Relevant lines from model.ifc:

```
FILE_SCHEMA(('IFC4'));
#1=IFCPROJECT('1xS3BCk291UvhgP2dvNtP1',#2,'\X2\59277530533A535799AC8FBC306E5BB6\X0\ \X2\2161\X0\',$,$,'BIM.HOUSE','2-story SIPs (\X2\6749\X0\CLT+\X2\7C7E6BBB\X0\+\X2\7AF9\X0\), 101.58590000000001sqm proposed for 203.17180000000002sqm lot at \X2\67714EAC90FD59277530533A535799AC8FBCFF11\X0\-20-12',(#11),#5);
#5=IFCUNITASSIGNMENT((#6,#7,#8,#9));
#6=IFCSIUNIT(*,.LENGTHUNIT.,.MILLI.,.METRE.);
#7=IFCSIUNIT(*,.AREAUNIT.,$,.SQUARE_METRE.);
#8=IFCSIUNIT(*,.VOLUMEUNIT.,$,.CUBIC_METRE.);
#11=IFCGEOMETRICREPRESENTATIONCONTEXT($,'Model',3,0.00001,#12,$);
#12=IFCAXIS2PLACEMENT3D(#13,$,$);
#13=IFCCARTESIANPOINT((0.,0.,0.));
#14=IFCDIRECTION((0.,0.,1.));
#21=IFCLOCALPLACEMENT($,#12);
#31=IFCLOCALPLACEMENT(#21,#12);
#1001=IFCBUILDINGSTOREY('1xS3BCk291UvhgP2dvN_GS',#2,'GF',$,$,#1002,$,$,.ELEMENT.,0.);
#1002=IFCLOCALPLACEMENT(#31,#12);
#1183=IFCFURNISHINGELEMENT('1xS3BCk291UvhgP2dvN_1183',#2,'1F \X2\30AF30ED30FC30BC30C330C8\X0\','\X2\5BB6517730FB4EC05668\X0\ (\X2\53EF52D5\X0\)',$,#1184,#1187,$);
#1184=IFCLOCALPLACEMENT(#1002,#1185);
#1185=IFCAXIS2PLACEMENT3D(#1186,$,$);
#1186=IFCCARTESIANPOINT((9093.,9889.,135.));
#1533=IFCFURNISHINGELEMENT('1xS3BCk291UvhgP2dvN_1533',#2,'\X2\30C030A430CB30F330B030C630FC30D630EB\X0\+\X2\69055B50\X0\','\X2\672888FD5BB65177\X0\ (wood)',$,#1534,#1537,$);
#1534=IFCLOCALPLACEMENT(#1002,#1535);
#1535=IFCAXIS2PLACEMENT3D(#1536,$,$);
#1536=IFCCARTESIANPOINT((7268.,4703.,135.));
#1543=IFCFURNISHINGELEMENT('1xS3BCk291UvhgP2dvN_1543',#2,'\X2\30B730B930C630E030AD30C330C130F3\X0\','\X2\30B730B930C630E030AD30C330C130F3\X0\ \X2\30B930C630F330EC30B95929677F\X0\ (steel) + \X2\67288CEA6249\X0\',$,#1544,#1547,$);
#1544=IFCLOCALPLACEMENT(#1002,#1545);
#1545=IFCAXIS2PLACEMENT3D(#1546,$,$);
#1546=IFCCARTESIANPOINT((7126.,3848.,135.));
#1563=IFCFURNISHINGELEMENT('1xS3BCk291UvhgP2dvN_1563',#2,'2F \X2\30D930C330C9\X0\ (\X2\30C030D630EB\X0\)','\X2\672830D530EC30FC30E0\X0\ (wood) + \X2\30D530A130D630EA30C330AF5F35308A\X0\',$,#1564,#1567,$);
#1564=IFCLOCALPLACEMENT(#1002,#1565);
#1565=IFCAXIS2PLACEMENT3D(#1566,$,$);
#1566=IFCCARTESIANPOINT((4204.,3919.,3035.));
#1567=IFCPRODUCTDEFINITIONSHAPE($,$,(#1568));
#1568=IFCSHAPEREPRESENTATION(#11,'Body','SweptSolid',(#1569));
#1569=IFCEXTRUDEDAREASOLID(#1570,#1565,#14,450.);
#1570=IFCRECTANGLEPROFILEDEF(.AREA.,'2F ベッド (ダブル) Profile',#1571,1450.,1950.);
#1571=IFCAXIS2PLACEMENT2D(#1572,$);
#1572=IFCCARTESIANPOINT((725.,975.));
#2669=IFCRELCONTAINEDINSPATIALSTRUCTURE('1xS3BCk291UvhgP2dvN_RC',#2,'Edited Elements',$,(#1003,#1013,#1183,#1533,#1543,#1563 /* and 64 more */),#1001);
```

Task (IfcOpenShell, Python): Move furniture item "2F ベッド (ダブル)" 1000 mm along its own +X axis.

```python
import ifcopenshell
import ifcopenshell.api.geometry
import ifcopenshell.util.placement

model = ifcopenshell.open("model.ifc")

item = model.by_guid("1xS3BCk291UvhgP2dvN_1563")
matrix = ifcopenshell.util.placement.get_local_placement(item.ObjectPlacement)
matrix[:3, 3] += matrix[:3, 0] * 1000.0
ifcopenshell.api.geometry.edit_object_placement(model, product=item, matrix=matrix, is_si=False)

print(ifcopenshell.util.placement.get_local_placement(item.ObjectPlacement).round(3) + 0.0)

model.write("model_v2.ifc")
```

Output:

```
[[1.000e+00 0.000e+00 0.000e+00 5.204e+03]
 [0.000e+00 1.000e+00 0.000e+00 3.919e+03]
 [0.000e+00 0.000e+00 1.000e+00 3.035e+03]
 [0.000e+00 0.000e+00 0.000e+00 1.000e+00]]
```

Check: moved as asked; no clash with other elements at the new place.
